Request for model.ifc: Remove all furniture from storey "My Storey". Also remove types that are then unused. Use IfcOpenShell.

First a look at what the model holds.

```python
import ifcopenshell
import ifcopenshell.util.element

model = ifcopenshell.open("model.ifc")
print(model.schema)
storey = next(s for s in model.by_type("IfcBuildingStorey") if s.Name == "My Storey")
furniture = [e for e in ifcopenshell.util.element.get_decomposition(storey) if e.is_a("IfcFurnishingElement")]
seen = {}
for e in furniture:
    element_type = ifcopenshell.util.element.get_type(e)
    name = element_type.Name if element_type not in (None, e) else None
    seen[name] = seen.get(name, 0) + 1
for name, count in sorted(seen.items(), key=str):
    print(count, "x", name)
```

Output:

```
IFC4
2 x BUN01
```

```python
import ifcopenshell
import ifcopenshell.api.root
import ifcopenshell.util.element

model = ifcopenshell.open("model.ifc")

storey = next(s for s in model.by_type("IfcBuildingStorey") if s.Name == "My Storey")
furniture = [e for e in ifcopenshell.util.element.get_decomposition(storey) if e.is_a("IfcFurnishingElement")]
types = {ifcopenshell.util.element.get_type(e) for e in furniture} - {None, *furniture}

for e in furniture:
    ifcopenshell.api.root.remove_product(model, product=e)
print(len(furniture), "removed")

unused = [t for t in types if not ifcopenshell.util.element.get_types(t)]
for t in unused:
    ifcopenshell.api.root.remove_product(model, product=t)
print(len(unused), "unused types removed")

model.write("model_v2.ifc")
```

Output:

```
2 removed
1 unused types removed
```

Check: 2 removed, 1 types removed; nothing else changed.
